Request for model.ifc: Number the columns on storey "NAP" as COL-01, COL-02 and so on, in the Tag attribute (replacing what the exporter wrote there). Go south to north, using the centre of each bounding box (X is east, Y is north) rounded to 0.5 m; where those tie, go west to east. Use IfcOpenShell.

First a look at what the model holds.

```python
import ifcopenshell
import ifcopenshell.util.element
import ifcopenshell.util.placement

model = ifcopenshell.open("model.ifc")
print(model.schema)
storey = next(s for s in model.by_type("IfcBuildingStorey") if s.Name == "NAP")
columns = [e for e in ifcopenshell.util.element.get_decomposition(storey) if e.is_a("IfcColumn")]
for e in sorted(columns, key=lambda e: e.id()):
    origin = ifcopenshell.util.placement.get_local_placement(e.ObjectPlacement)[:3, 3]
    print(e.id(), e.Tag, e.Name, origin.round(2) + 0.0, sep=" | ")
```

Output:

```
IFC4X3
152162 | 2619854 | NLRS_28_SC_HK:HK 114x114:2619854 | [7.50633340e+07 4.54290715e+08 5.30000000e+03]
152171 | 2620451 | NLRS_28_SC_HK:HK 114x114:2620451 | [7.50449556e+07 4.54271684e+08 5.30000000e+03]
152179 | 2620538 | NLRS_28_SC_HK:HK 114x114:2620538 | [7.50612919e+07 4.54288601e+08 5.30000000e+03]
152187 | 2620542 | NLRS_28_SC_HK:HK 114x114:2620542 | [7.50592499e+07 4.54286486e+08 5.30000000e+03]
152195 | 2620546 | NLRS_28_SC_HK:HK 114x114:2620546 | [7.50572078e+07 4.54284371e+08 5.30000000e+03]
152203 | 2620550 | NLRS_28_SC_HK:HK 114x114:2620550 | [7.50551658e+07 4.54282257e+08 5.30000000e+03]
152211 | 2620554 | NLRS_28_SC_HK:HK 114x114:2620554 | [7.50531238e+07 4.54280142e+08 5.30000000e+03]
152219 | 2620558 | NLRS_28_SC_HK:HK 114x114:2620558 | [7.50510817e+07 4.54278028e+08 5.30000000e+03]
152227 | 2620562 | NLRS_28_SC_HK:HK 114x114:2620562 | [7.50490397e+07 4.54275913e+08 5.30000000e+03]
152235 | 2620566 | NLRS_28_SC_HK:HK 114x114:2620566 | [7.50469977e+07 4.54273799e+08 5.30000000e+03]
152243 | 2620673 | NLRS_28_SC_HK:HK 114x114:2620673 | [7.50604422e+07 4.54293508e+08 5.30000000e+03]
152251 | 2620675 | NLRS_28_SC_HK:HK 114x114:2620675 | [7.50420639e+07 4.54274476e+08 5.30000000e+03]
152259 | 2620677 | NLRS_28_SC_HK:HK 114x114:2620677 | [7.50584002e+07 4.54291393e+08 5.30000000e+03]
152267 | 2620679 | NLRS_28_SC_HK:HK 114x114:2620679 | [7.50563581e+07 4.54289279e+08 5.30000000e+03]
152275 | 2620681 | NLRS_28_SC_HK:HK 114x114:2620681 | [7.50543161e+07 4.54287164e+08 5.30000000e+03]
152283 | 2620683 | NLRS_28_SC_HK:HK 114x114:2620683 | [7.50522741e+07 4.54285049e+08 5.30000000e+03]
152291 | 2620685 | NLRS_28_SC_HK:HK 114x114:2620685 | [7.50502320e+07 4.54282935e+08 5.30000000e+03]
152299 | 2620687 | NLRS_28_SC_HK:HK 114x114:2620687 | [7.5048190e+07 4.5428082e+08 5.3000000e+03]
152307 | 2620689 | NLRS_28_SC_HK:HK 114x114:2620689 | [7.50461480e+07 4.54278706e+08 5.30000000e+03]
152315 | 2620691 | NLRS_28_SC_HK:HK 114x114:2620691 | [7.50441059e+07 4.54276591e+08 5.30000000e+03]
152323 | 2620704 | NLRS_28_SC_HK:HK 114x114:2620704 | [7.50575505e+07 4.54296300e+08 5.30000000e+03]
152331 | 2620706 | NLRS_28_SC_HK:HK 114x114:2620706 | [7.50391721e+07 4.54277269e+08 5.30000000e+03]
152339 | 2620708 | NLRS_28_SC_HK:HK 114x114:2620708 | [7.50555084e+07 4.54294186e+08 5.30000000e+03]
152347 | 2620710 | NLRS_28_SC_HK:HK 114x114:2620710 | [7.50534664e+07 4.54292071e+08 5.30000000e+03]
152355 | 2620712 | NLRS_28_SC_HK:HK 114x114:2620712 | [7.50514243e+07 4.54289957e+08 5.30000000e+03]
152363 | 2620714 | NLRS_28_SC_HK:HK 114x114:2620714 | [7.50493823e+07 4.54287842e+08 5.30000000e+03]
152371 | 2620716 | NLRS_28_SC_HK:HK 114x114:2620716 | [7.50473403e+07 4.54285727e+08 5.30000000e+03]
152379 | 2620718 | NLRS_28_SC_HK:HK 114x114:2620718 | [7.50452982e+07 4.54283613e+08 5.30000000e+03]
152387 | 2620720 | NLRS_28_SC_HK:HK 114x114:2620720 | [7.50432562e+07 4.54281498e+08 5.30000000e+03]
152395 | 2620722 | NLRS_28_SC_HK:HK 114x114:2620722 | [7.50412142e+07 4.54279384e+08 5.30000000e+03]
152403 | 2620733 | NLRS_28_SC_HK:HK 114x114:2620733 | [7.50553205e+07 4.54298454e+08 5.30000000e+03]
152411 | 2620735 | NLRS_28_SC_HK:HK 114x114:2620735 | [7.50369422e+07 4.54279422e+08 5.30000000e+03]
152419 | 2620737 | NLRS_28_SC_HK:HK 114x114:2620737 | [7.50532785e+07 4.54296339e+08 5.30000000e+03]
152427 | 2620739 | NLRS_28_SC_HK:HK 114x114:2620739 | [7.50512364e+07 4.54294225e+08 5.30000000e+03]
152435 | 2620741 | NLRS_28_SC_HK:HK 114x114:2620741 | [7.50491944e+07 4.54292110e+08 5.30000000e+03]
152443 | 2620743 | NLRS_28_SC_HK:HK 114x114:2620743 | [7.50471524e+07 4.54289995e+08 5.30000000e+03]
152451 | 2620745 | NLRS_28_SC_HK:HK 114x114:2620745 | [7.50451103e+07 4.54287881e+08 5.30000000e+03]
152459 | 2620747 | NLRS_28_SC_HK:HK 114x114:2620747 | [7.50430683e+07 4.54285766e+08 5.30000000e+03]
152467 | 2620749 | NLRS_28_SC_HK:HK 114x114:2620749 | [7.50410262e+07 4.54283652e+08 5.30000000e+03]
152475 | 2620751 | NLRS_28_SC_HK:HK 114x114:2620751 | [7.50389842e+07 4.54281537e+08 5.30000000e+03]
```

```python
import ifcopenshell
import ifcopenshell.geom
import ifcopenshell.util.element
import ifcopenshell.util.shape

model = ifcopenshell.open("model.ifc")
settings = ifcopenshell.geom.settings()
settings.set("use-world-coords", True)


def centre(element):
    shape = ifcopenshell.geom.create_shape(settings, element)
    return ifcopenshell.util.shape.get_bbox_centroid(shape.geometry)


storey = next(s for s in model.by_type("IfcBuildingStorey") if s.Name == "NAP")
columns = [e for e in ifcopenshell.util.element.get_decomposition(storey) if e.is_a("IfcColumn")]

# Insertion points can sit at a corner or the storey origin, so sort by the geometry (in metres).
centres = {e: centre(e) for e in columns}
columns.sort(key=lambda e: (round(centres[e][1] / 0.5), centres[e][0]))

for i, e in enumerate(columns, start=1):
    number = f"COL-{i:02d}"
    e.Tag = number
    print(e.id(), number)

model.write("model_edited.ifc")
```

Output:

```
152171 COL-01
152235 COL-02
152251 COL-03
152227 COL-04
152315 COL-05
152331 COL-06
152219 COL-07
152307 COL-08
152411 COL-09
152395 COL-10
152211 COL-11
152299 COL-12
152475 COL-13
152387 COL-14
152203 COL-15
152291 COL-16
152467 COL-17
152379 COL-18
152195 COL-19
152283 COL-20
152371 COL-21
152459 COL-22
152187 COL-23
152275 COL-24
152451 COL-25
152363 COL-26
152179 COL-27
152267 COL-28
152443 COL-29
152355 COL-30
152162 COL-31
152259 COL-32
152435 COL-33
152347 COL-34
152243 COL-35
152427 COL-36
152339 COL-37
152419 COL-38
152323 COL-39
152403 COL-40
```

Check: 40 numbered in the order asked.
